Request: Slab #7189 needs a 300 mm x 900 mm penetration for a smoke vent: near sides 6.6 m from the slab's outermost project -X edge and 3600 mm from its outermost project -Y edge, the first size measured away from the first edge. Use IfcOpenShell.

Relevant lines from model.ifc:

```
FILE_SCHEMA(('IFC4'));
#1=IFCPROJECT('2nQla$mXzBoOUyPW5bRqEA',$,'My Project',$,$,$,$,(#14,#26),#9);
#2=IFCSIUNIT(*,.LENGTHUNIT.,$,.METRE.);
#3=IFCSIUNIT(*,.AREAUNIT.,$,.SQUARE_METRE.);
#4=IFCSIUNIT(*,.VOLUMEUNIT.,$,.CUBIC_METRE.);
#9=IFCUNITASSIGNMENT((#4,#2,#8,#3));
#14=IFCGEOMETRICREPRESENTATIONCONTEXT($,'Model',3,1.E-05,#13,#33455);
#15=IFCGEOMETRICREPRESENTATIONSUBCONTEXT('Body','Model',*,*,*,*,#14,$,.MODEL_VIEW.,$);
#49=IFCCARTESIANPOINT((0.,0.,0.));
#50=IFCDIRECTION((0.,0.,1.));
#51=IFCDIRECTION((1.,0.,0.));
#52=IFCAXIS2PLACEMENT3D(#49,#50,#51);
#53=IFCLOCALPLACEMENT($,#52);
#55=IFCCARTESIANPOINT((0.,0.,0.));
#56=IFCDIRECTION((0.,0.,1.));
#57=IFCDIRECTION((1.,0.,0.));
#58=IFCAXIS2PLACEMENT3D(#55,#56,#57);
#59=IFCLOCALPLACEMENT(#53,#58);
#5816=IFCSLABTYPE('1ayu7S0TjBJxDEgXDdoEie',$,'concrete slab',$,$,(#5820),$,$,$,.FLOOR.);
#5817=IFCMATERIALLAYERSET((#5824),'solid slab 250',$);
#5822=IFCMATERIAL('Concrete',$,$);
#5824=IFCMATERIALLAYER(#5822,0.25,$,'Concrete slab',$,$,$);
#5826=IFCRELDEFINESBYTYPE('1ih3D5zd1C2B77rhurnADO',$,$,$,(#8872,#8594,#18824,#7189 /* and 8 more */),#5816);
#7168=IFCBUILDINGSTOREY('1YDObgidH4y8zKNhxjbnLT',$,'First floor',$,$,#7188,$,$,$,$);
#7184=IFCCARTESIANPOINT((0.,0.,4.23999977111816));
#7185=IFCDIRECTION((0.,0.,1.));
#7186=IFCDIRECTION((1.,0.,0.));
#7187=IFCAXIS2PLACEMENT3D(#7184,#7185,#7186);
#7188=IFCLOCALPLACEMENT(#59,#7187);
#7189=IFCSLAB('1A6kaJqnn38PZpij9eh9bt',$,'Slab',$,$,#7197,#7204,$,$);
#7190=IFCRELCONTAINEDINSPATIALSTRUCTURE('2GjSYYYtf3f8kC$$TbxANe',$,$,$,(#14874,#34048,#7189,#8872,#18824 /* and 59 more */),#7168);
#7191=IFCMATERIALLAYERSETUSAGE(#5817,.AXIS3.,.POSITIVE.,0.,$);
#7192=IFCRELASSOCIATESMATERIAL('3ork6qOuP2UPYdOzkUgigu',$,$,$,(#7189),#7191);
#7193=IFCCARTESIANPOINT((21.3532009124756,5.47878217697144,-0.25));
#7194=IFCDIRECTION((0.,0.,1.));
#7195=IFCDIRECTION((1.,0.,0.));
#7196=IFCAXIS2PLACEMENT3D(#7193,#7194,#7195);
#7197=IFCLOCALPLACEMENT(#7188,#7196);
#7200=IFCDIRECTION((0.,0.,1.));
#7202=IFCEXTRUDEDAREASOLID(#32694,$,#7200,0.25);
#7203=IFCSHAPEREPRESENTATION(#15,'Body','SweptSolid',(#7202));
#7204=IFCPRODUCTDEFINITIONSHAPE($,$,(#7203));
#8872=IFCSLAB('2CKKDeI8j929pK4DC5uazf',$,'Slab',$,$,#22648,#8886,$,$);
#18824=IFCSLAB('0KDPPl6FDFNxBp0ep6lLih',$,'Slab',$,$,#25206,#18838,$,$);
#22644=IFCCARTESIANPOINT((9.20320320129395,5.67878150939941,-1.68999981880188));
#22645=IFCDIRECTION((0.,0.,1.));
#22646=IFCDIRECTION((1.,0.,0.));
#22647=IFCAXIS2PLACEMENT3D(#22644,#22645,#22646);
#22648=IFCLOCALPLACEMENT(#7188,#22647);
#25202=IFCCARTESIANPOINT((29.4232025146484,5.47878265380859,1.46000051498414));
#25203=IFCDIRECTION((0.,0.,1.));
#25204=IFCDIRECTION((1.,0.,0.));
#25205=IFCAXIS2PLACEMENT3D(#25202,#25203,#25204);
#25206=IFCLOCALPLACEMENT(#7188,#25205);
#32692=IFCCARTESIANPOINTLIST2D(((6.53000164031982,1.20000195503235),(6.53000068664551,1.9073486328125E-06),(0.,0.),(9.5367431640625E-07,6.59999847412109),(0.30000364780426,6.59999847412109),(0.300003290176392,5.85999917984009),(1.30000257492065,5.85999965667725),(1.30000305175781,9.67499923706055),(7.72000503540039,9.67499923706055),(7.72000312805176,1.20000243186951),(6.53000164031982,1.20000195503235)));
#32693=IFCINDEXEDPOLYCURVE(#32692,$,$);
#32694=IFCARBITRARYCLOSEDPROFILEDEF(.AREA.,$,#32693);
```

```python
import numpy as np
import ifcopenshell
import ifcopenshell.api.feature
import ifcopenshell.api.geometry
import ifcopenshell.api.root
import ifcopenshell.geom
import ifcopenshell.util.placement
import ifcopenshell.util.representation
import ifcopenshell.util.shape
import ifcopenshell.util.unit

model = ifcopenshell.open("model.ifc")
unit_scale = ifcopenshell.util.unit.calculate_unit_scale(model)
settings = ifcopenshell.geom.settings()


def volume(element):
    """Net volume in cubic metres, openings subtracted."""
    shape = ifcopenshell.geom.create_shape(settings, element)
    return ifcopenshell.util.shape.get_volume(shape.geometry)


slab = model.by_guid("1A6kaJqnn38PZpij9eh9bt")
before = volume(slab)

# Extent in the slab's own axes, in metres. The edges named are its -X and -Y sides.
slab_shape = ifcopenshell.geom.create_shape(settings, slab)
vertices = ifcopenshell.util.shape.get_vertices(slab_shape.geometry)
x_min, y_min, bottom = vertices.min(axis=0)
top = vertices[:, 2].max()

opening = ifcopenshell.api.root.create_entity(model, ifc_class="IfcOpeningElement", name="Smoke vent opening", predefined_type="OPENING")
context = ifcopenshell.util.representation.get_context(model, "Model", "Body", "MODEL_VIEW")
width, depth = 0.3, 0.9
outline = [(0.0, 0.0), (width, 0.0), (width, depth), (0.0, depth), (0.0, 0.0)]
# Overshoot both faces by 50 mm so the cut is clean.
shape = ifcopenshell.api.geometry.add_slab_representation(
    model, context=context, depth=top - bottom + 0.1, polyline=outline
)
ifcopenshell.api.geometry.assign_representation(model, product=opening, representation=shape)

matrix = ifcopenshell.util.placement.get_local_placement(slab.ObjectPlacement)
matrix[:, 3] = matrix @ np.append(np.array([x_min + 6.6, y_min + 3.6, bottom - 0.05]) / unit_scale, 1.0)
ifcopenshell.api.geometry.edit_object_placement(model, product=opening, matrix=matrix, is_si=False)
ifcopenshell.api.feature.add_feature(model, feature=opening, element=slab)

after = volume(slab)

print(f"slab volume {before:.3f} -> {after:.3f} m3")

model.write("model_edited.ifc")
```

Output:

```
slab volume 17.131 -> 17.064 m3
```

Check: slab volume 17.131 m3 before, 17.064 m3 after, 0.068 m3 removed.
